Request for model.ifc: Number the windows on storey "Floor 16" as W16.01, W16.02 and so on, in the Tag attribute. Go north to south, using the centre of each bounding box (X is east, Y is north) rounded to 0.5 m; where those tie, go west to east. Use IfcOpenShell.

First a look at what the model holds.

```python
import ifcopenshell
import ifcopenshell.util.element
import ifcopenshell.util.placement

model = ifcopenshell.open("model.ifc")
print(model.schema)
storey = next(s for s in model.by_type("IfcBuildingStorey") if s.Name == "Floor 16")
windows = [e for e in ifcopenshell.util.element.get_decomposition(storey) if e.is_a("IfcWindow")]
for e in sorted(windows, key=lambda e: e.id()):
    origin = ifcopenshell.util.placement.get_local_placement(e.ObjectPlacement)[:3, 3]
    print(e.id(), e.Tag, e.Name, origin.round(2) + 0.0, sep=" | ")
```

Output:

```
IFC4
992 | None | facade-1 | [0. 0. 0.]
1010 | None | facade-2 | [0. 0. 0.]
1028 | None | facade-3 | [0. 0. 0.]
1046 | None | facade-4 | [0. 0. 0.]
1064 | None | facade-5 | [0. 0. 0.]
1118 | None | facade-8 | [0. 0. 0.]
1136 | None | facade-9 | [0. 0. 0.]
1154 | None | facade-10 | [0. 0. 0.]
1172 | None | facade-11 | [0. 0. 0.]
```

```python
import ifcopenshell
import ifcopenshell.geom
import ifcopenshell.util.element
import ifcopenshell.util.shape

model = ifcopenshell.open("model.ifc")
settings = ifcopenshell.geom.settings()
settings.set("use-world-coords", True)


def centre(element):
    shape = ifcopenshell.geom.create_shape(settings, element)
    return ifcopenshell.util.shape.get_bbox_centroid(shape.geometry)


storey = next(s for s in model.by_type("IfcBuildingStorey") if s.Name == "Floor 16")
windows = [e for e in ifcopenshell.util.element.get_decomposition(storey) if e.is_a("IfcWindow")]

# Insertion points can sit at a corner or the storey origin, so sort by the geometry (in metres).
centres = {e: centre(e) for e in windows}
windows.sort(key=lambda e: (-round(centres[e][1] / 0.5), centres[e][0]))

for i, e in enumerate(windows, start=1):
    number = f"W16.{i:02d}"
    e.Tag = number
    print(e.id(), number)

model.write("model_rev.ifc")
```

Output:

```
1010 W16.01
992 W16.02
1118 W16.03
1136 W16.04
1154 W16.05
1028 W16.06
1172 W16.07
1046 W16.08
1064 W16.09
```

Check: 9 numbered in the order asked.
